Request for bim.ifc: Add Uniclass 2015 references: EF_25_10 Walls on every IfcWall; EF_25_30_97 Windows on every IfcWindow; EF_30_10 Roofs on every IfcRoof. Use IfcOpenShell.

First a look at what the model holds.

```python
import ifcopenshell

model = ifcopenshell.open("bim.ifc")
print(model.schema)
print("classifications:", [c.Name for c in model.by_type("IfcClassification")])
for ifc_class in ("IfcDoor", "IfcRoof", "IfcStair", "IfcWall", "IfcWindow"):
    print(ifc_class, len(model.by_type(ifc_class)))
```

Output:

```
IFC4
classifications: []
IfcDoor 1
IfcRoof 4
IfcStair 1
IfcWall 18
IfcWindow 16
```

```python
import ifcopenshell
import ifcopenshell.api.classification

model = ifcopenshell.open("bim.ifc")

system = ifcopenshell.api.classification.add_classification(model, classification="Uniclass 2015")

codes = {
    "IfcWall": ("EF_25_10", "Walls"),
    "IfcWindow": ("EF_25_30_97", "Windows"),
    "IfcRoof": ("EF_30_10", "Roofs"),
}
for ifc_class, (code, name) in codes.items():
    products = model.by_type(ifc_class)
    ifcopenshell.api.classification.add_reference(
        model, products=products, classification=system, identification=code, name=name
    )
    print(code, len(products))

model.write("bim-out.ifc")
```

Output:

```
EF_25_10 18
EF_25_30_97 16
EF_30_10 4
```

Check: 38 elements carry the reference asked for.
